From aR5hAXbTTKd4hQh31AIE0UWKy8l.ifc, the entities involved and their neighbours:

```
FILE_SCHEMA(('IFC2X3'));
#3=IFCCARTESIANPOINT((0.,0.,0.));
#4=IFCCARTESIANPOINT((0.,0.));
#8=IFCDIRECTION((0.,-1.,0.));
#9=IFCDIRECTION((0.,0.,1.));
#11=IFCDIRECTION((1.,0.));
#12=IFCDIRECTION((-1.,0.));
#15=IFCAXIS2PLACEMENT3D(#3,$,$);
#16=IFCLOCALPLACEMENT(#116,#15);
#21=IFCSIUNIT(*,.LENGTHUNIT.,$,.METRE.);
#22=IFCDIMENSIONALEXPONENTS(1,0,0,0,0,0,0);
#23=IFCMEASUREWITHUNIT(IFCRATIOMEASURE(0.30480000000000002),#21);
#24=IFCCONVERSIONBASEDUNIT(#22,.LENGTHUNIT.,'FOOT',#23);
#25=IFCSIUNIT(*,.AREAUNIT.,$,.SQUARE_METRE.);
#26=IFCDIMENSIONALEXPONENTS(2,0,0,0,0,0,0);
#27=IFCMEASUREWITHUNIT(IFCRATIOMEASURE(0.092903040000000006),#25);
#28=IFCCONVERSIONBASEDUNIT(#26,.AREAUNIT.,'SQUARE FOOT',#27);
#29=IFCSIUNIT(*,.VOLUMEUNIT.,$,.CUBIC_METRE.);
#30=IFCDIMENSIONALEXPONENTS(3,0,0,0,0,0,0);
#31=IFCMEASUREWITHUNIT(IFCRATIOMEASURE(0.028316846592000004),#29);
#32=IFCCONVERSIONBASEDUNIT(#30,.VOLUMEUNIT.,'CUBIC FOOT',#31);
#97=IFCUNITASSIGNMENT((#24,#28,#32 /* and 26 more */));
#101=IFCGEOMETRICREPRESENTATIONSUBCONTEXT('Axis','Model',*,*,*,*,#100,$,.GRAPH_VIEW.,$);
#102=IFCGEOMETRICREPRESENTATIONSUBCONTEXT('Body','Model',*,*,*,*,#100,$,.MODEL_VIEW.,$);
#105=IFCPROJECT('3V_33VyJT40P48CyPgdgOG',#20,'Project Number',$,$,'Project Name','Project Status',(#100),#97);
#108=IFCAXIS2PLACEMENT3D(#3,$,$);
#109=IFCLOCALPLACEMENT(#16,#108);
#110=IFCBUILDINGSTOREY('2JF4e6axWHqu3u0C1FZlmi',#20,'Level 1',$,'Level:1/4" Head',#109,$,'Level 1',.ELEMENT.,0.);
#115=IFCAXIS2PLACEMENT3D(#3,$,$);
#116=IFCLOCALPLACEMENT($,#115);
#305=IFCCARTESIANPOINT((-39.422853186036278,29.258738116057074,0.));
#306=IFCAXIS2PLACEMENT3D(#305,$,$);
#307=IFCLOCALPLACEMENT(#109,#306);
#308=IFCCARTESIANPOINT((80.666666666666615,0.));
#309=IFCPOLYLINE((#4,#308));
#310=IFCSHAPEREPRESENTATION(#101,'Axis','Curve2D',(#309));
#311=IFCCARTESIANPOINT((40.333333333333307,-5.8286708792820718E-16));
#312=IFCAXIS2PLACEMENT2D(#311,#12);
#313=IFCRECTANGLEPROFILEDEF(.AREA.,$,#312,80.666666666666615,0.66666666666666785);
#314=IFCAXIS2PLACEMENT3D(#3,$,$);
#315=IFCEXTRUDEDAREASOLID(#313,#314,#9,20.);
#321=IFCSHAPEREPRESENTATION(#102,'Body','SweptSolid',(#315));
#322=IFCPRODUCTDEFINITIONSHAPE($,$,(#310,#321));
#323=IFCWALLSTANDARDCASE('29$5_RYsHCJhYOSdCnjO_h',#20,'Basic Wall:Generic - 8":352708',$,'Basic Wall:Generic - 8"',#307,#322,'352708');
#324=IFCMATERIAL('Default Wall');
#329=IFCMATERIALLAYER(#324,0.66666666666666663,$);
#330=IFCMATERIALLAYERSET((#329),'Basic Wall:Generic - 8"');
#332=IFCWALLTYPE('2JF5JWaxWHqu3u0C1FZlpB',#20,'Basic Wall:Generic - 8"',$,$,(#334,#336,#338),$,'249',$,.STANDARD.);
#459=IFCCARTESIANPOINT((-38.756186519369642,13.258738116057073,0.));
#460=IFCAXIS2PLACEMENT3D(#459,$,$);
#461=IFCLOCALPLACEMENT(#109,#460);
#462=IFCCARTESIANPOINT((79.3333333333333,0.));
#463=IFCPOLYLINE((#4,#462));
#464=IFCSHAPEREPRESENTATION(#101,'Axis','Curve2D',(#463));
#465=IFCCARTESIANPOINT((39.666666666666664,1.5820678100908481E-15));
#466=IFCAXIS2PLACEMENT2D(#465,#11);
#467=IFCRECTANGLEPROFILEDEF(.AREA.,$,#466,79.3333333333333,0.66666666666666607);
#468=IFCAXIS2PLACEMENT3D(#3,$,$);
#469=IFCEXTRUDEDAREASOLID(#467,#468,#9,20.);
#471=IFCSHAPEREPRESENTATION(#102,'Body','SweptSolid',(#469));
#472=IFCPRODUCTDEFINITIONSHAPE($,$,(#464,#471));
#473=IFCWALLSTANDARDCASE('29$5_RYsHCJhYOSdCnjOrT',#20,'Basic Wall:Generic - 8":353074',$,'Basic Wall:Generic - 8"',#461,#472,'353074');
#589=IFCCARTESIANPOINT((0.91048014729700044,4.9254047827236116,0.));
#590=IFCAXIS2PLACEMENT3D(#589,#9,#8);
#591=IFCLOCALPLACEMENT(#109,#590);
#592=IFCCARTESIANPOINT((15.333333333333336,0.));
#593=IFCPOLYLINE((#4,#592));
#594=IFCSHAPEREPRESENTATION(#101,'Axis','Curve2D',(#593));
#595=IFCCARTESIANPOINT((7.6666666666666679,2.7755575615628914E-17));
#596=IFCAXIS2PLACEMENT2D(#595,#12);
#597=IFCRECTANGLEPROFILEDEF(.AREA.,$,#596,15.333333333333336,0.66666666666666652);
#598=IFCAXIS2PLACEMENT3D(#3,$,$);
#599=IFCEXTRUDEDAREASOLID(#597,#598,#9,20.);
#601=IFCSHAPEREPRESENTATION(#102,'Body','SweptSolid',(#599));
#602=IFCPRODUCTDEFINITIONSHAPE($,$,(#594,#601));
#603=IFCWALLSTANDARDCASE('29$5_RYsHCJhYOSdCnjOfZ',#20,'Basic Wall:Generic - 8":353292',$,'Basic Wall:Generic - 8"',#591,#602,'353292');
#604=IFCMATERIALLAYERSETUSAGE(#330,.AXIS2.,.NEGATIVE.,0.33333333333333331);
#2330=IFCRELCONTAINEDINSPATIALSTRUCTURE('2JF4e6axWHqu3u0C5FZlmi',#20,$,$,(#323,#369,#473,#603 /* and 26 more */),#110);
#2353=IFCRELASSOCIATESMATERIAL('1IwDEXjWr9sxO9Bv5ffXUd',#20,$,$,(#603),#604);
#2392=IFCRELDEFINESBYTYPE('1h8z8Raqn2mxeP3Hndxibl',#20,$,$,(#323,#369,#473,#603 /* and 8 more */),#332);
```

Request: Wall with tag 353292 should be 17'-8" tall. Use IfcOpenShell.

```python
import ifcopenshell
import ifcopenshell.geom
import ifcopenshell.util.representation
import ifcopenshell.util.shape
import ifcopenshell.util.unit

model = ifcopenshell.open("aR5hAXbTTKd4hQh31AIE0UWKy8l.ifc")
unit_scale = ifcopenshell.util.unit.calculate_unit_scale(model)
settings = ifcopenshell.geom.settings()


def volume(element):
    """Net volume in cubic metres, openings subtracted."""
    shape = ifcopenshell.geom.create_shape(settings, element)
    return ifcopenshell.util.shape.get_volume(shape.geometry)


wall = model.by_guid("29$5_RYsHCJhYOSdCnjOfZ")
before = volume(wall)

body = ifcopenshell.util.representation.get_representation(wall, "Model", "Body")
solid = body.Items[0]
old_height = solid.Depth
solid.Depth = 212 * 0.0254 / unit_scale
after = volume(wall)

print(f"height {old_height:g} -> {solid.Depth:g}, volume {before:.3f} -> {after:.3f} m3")

model.write("aR5hAXbTTKd4hQh31AIE0UWKy8l_rev.ifc")
```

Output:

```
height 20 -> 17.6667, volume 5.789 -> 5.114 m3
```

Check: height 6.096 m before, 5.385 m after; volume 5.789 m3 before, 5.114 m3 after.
